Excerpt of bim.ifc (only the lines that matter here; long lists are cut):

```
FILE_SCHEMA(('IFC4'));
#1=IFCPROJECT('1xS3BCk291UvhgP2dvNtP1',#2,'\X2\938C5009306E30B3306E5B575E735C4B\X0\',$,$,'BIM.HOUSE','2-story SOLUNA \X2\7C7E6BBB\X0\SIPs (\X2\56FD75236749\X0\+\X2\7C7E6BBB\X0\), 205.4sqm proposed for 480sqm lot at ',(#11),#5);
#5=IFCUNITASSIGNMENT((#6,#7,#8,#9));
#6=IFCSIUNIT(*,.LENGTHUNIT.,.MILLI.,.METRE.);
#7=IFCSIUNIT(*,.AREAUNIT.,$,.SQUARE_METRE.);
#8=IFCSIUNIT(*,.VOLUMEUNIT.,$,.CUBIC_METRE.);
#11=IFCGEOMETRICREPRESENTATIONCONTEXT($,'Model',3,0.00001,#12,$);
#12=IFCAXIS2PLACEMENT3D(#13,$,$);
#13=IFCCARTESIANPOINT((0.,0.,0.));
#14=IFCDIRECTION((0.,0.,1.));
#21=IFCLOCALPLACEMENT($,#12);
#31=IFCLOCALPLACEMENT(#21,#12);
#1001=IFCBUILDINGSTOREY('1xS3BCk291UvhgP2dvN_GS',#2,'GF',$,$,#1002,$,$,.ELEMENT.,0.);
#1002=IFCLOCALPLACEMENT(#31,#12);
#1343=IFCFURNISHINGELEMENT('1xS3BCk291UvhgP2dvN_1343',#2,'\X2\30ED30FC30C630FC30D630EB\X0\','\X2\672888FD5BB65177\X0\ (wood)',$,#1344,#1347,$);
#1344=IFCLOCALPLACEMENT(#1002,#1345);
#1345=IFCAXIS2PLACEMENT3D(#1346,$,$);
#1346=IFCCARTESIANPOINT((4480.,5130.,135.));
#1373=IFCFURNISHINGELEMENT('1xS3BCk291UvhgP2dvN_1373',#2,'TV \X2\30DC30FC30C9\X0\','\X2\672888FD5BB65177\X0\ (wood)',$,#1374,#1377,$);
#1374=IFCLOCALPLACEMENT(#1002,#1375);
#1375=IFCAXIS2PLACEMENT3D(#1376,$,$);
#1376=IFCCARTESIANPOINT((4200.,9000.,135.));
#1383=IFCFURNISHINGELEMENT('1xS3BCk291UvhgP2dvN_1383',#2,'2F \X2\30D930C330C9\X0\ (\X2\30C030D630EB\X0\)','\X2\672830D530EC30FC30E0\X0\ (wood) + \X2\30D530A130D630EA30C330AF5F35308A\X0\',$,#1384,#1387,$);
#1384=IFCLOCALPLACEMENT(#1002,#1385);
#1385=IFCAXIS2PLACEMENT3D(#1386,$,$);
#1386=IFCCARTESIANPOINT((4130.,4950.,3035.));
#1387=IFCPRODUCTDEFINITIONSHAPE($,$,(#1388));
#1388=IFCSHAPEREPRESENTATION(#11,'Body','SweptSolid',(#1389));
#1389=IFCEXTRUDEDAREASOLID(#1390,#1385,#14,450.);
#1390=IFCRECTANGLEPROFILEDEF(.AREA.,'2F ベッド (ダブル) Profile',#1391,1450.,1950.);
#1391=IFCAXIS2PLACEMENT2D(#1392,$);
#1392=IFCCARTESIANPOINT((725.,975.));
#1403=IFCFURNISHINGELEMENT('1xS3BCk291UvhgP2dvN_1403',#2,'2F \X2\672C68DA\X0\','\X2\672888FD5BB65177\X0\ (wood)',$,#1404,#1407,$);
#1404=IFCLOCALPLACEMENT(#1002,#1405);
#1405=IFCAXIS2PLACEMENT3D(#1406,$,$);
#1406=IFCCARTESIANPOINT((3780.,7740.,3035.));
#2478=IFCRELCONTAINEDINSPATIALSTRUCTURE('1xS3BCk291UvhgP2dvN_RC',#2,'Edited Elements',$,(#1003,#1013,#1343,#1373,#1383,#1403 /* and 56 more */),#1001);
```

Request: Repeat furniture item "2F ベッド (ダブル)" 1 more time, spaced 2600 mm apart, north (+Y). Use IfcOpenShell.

```python
import numpy as np
import ifcopenshell
import ifcopenshell.api.geometry
import ifcopenshell.api.root
import ifcopenshell.util.element
import ifcopenshell.util.placement
import ifcopenshell.util.unit

model = ifcopenshell.open("bim.ifc")
unit_scale = ifcopenshell.util.unit.calculate_unit_scale(model)


def reuse_history(source, copy):
    """copy_class also copies each property set's owner history, people and application; keep the originals."""
    for rel in copy.IsDefinedBy:
        if rel.is_a("IfcRelDefinesByProperties") and (history := rel.RelatingPropertyDefinition.OwnerHistory):
            rel.RelatingPropertyDefinition.OwnerHistory = source.OwnerHistory
            ifcopenshell.util.element.remove_deep2(model, history)


source = model.by_id(1383)
base = ifcopenshell.util.placement.get_local_placement(source.ObjectPlacement)
step = np.array([0.0, 1.0, 0.0]) * 2.6 / unit_scale

for i in range(1, 2):
    copy = ifcopenshell.api.root.copy_class(model, product=source)
    copy.Representation = ifcopenshell.util.element.copy_deep(
        model, source.Representation, exclude=["IfcGeometricRepresentationContext", "IfcRepresentationMap"]
    )
    reuse_history(source, copy)
    matrix = base.copy()
    matrix[:3, 3] += i * step
    print("added at", matrix[:3, 3].round(3) + 0.0)
    ifcopenshell.api.geometry.edit_object_placement(model, product=copy, matrix=matrix, is_si=False)

model.write("bim-out.ifc")
```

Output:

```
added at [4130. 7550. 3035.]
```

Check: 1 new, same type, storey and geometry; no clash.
